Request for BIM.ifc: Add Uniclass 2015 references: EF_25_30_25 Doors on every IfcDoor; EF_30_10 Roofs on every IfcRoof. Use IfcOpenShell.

First a look at what the model holds.

```python
import ifcopenshell

model = ifcopenshell.open("BIM.ifc")
print(model.schema)
print("classifications:", [c.Name for c in model.by_type("IfcClassification")])
for ifc_class in ("IfcDoor", "IfcRoof", "IfcStair", "IfcWall", "IfcWindow"):
    print(ifc_class, len(model.by_type(ifc_class)))
```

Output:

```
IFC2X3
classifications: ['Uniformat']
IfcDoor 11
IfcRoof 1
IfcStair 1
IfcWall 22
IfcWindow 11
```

```python
import ifcopenshell
import ifcopenshell.api.classification

model = ifcopenshell.open("BIM.ifc")

# IFC2X3 requires Source and Edition and has no link from the project to the system.
system = model.create_entity("IfcClassification", Source="NBS", Edition="2015", Name="Uniclass 2015")

codes = {
    "IfcDoor": ("EF_25_30_25", "Doors"),
    "IfcRoof": ("EF_30_10", "Roofs"),
}
for ifc_class, (code, name) in codes.items():
    products = model.by_type(ifc_class)
    ifcopenshell.api.classification.add_reference(
        model, products=products, classification=system, identification=code, name=name
    )
    print(code, len(products))

model.write("BIM_updated.ifc")
```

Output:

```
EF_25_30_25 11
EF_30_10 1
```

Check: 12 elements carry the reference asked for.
